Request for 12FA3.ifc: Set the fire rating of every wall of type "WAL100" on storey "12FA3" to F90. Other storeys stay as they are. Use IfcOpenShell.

First a look at what the model holds.

```python
import ifcopenshell
import ifcopenshell.util.element

model = ifcopenshell.open("12FA3.ifc")
print(model.schema)
storey = next(s for s in model.by_type("IfcBuildingStorey") if s.Name == "12FA3")
walls = [e for e in ifcopenshell.util.element.get_decomposition(storey) if e.is_a("IfcWall")]
seen = {}
for e in walls:
    element_type = ifcopenshell.util.element.get_type(e)
    key = (element_type.Name if element_type != e and element_type else None, ifcopenshell.util.element.get_pset(e, "Pset_WallCommon", "FireRating"))
    seen[key] = seen.get(key, 0) + 1
for (name, value), count in sorted(seen.items(), key=str):
    print(count, "x", name, "|", value)
```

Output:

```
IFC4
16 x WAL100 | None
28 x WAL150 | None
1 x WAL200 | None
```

```python
import ifcopenshell
import ifcopenshell.api.pset
import ifcopenshell.util.element

model = ifcopenshell.open("12FA3.ifc")

storey = next(s for s in model.by_type("IfcBuildingStorey") if s.Name == "12FA3")
walls = [e for e in ifcopenshell.util.element.get_decomposition(storey) if e.is_a("IfcWall")]

count = 0
for e in walls:
    element_type = ifcopenshell.util.element.get_type(e)
    if element_type in (None, e) or element_type.Name != "WAL100":
        continue
    # add_pset returns the element's existing set when there is one.
    pset = ifcopenshell.api.pset.add_pset(model, product=e, name="Pset_WallCommon")
    ifcopenshell.api.pset.edit_pset(model, pset=pset, properties={"FireRating": "F90"})
    count += 1

print(count, "walls updated")

model.write("12FA3_edited.ifc")
```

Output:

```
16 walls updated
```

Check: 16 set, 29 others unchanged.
